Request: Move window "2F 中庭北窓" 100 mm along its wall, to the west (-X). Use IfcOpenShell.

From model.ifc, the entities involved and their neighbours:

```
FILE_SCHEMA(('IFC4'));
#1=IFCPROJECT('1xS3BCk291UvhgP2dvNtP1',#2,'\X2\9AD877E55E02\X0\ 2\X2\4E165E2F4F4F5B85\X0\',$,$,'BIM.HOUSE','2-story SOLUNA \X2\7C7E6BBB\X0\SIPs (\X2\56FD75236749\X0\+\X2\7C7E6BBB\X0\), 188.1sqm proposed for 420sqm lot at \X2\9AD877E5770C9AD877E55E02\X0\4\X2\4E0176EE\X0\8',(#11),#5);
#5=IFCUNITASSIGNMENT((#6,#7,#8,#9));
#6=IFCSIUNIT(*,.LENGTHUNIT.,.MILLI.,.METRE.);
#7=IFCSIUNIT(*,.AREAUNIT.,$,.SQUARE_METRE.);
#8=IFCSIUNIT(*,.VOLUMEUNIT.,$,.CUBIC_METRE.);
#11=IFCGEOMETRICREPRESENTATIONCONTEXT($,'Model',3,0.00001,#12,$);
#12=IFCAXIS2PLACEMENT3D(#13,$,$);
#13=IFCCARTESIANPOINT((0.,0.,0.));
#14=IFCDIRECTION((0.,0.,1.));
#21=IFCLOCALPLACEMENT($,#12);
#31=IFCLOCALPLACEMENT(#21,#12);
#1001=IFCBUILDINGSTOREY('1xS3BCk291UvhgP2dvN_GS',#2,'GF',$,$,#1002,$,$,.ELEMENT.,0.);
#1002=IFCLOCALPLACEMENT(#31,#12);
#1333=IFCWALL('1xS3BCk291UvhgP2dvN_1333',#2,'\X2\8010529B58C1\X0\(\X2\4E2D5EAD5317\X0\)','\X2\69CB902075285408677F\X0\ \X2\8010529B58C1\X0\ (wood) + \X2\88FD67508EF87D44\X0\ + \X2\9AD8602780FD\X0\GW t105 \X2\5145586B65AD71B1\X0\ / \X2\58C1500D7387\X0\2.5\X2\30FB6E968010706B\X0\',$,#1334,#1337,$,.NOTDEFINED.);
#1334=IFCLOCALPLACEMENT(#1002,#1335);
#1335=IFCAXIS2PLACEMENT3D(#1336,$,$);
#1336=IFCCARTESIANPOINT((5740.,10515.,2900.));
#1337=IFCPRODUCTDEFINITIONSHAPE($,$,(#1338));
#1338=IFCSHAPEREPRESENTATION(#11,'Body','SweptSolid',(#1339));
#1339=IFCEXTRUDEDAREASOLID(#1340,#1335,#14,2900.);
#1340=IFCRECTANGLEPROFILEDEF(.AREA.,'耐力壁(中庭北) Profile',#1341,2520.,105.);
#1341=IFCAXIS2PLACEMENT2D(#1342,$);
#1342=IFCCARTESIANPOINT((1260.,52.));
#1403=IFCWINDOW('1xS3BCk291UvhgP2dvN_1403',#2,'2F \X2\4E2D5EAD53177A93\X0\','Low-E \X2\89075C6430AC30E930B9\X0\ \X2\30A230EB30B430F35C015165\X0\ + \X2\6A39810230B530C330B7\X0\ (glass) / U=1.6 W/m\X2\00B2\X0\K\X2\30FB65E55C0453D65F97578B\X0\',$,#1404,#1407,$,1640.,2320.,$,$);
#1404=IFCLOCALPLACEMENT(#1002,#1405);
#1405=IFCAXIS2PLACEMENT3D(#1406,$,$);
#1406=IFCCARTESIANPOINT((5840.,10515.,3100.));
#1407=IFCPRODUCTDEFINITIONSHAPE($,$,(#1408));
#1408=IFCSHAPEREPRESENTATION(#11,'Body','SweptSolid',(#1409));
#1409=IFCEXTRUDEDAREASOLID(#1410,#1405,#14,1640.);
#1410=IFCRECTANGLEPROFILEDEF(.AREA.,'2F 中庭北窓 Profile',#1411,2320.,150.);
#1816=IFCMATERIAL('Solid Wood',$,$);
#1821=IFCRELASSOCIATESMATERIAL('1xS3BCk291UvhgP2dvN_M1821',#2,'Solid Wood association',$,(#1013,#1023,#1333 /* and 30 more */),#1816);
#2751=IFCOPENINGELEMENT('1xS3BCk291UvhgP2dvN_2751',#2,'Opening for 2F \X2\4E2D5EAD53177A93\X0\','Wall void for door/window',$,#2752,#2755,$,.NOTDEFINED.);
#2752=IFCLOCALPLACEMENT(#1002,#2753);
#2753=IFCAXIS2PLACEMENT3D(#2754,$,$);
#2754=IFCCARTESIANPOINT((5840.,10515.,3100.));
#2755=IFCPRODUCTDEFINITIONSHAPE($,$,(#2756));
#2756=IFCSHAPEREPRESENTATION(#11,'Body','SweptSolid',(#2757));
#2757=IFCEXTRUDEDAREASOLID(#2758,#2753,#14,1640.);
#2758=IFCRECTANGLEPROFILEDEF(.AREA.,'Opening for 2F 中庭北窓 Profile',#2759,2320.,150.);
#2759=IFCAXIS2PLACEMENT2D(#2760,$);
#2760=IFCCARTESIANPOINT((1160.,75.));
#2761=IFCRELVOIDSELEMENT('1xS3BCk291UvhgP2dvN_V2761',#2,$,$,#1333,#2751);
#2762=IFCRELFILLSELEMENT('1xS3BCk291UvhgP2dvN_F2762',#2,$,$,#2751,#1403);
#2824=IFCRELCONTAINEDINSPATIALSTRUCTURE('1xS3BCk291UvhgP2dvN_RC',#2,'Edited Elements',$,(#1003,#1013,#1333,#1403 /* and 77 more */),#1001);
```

```python
import ifcopenshell
import ifcopenshell.api.geometry
import ifcopenshell.util.placement

model = ifcopenshell.open("model.ifc")

window = model.by_id(1403)
opening = window.FillsVoids[0].RelatingOpeningElement
wall = opening.VoidsElements[0].RelatingBuildingElement

wall_matrix = ifcopenshell.util.placement.get_local_placement(wall.ObjectPlacement)
shift = wall_matrix[:3, 0] * -100.0
before = ifcopenshell.util.placement.get_local_placement(window.ObjectPlacement)[:3, 3].copy()

# The window is not placed relative to its opening, so move both.
for product in (opening, window):
    matrix = ifcopenshell.util.placement.get_local_placement(product.ObjectPlacement)
    matrix[:3, 3] += shift
    ifcopenshell.api.geometry.edit_object_placement(model, product=product, matrix=matrix, is_si=False)

after = ifcopenshell.util.placement.get_local_placement(window.ObjectPlacement)[:3, 3]
print("window moved by", (after - before).round(3) + 0.0)

model.write("model_v2.ifc")
```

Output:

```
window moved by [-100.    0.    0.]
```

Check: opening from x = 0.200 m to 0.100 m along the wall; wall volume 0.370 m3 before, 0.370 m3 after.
